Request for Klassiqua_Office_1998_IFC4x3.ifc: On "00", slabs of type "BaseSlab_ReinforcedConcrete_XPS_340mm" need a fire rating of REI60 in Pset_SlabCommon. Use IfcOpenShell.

First a look at what the model holds.

```python
import ifcopenshell
import ifcopenshell.util.element

model = ifcopenshell.open("Klassiqua_Office_1998_IFC4x3.ifc")
print(model.schema)
storey = next(s for s in model.by_type("IfcBuildingStorey") if s.Name == "00")
slabs = [e for e in ifcopenshell.util.element.get_decomposition(storey) if e.is_a("IfcSlab")]
seen = {}
for e in slabs:
    element_type = ifcopenshell.util.element.get_type(e)
    key = (element_type.Name if element_type != e and element_type else None, ifcopenshell.util.element.get_pset(e, "Pset_SlabCommon", "FireRating"))
    seen[key] = seen.get(key, 0) + 1
for (name, value), count in sorted(seen.items(), key=str):
    print(count, "x", name, "|", value)
```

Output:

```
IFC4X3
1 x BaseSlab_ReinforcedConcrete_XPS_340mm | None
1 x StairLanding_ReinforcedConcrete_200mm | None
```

```python
import ifcopenshell
import ifcopenshell.api.pset
import ifcopenshell.util.element

model = ifcopenshell.open("Klassiqua_Office_1998_IFC4x3.ifc")

storey = next(s for s in model.by_type("IfcBuildingStorey") if s.Name == "00")
slabs = [e for e in ifcopenshell.util.element.get_decomposition(storey) if e.is_a("IfcSlab")]

count = 0
for e in slabs:
    element_type = ifcopenshell.util.element.get_type(e)
    if element_type in (None, e) or element_type.Name != "BaseSlab_ReinforcedConcrete_XPS_340mm":
        continue
    # add_pset returns the element's existing set when there is one.
    pset = ifcopenshell.api.pset.add_pset(model, product=e, name="Pset_SlabCommon")
    ifcopenshell.api.pset.edit_pset(model, pset=pset, properties={"FireRating": "REI60"})
    count += 1

print(count, "slabs updated")

model.write("Klassiqua_Office_1998_IFC4x3_edited.ifc")
```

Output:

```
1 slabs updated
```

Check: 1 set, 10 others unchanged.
